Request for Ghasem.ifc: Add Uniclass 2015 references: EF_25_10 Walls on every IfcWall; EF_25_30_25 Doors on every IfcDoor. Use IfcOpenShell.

First a look at what the model holds.

```python
import ifcopenshell

model = ifcopenshell.open("Ghasem.ifc")
print(model.schema)
print("classifications:", [c.Name for c in model.by_type("IfcClassification")])
for ifc_class in ("IfcDoor", "IfcRoof", "IfcStair", "IfcWall", "IfcWindow"):
    print(ifc_class, len(model.by_type(ifc_class)))
```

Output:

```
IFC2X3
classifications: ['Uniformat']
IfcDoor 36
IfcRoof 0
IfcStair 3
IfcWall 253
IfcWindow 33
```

```python
import ifcopenshell
import ifcopenshell.api.classification

model = ifcopenshell.open("Ghasem.ifc")

# IFC2X3 requires Source and Edition and has no link from the project to the system.
system = model.create_entity("IfcClassification", Source="NBS", Edition="2015", Name="Uniclass 2015")

codes = {
    "IfcWall": ("EF_25_10", "Walls"),
    "IfcDoor": ("EF_25_30_25", "Doors"),
}
for ifc_class, (code, name) in codes.items():
    products = model.by_type(ifc_class)
    ifcopenshell.api.classification.add_reference(
        model, products=products, classification=system, identification=code, name=name
    )
    print(code, len(products))

model.write("Ghasem_updated.ifc")
```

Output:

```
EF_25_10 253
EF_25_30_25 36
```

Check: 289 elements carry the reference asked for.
